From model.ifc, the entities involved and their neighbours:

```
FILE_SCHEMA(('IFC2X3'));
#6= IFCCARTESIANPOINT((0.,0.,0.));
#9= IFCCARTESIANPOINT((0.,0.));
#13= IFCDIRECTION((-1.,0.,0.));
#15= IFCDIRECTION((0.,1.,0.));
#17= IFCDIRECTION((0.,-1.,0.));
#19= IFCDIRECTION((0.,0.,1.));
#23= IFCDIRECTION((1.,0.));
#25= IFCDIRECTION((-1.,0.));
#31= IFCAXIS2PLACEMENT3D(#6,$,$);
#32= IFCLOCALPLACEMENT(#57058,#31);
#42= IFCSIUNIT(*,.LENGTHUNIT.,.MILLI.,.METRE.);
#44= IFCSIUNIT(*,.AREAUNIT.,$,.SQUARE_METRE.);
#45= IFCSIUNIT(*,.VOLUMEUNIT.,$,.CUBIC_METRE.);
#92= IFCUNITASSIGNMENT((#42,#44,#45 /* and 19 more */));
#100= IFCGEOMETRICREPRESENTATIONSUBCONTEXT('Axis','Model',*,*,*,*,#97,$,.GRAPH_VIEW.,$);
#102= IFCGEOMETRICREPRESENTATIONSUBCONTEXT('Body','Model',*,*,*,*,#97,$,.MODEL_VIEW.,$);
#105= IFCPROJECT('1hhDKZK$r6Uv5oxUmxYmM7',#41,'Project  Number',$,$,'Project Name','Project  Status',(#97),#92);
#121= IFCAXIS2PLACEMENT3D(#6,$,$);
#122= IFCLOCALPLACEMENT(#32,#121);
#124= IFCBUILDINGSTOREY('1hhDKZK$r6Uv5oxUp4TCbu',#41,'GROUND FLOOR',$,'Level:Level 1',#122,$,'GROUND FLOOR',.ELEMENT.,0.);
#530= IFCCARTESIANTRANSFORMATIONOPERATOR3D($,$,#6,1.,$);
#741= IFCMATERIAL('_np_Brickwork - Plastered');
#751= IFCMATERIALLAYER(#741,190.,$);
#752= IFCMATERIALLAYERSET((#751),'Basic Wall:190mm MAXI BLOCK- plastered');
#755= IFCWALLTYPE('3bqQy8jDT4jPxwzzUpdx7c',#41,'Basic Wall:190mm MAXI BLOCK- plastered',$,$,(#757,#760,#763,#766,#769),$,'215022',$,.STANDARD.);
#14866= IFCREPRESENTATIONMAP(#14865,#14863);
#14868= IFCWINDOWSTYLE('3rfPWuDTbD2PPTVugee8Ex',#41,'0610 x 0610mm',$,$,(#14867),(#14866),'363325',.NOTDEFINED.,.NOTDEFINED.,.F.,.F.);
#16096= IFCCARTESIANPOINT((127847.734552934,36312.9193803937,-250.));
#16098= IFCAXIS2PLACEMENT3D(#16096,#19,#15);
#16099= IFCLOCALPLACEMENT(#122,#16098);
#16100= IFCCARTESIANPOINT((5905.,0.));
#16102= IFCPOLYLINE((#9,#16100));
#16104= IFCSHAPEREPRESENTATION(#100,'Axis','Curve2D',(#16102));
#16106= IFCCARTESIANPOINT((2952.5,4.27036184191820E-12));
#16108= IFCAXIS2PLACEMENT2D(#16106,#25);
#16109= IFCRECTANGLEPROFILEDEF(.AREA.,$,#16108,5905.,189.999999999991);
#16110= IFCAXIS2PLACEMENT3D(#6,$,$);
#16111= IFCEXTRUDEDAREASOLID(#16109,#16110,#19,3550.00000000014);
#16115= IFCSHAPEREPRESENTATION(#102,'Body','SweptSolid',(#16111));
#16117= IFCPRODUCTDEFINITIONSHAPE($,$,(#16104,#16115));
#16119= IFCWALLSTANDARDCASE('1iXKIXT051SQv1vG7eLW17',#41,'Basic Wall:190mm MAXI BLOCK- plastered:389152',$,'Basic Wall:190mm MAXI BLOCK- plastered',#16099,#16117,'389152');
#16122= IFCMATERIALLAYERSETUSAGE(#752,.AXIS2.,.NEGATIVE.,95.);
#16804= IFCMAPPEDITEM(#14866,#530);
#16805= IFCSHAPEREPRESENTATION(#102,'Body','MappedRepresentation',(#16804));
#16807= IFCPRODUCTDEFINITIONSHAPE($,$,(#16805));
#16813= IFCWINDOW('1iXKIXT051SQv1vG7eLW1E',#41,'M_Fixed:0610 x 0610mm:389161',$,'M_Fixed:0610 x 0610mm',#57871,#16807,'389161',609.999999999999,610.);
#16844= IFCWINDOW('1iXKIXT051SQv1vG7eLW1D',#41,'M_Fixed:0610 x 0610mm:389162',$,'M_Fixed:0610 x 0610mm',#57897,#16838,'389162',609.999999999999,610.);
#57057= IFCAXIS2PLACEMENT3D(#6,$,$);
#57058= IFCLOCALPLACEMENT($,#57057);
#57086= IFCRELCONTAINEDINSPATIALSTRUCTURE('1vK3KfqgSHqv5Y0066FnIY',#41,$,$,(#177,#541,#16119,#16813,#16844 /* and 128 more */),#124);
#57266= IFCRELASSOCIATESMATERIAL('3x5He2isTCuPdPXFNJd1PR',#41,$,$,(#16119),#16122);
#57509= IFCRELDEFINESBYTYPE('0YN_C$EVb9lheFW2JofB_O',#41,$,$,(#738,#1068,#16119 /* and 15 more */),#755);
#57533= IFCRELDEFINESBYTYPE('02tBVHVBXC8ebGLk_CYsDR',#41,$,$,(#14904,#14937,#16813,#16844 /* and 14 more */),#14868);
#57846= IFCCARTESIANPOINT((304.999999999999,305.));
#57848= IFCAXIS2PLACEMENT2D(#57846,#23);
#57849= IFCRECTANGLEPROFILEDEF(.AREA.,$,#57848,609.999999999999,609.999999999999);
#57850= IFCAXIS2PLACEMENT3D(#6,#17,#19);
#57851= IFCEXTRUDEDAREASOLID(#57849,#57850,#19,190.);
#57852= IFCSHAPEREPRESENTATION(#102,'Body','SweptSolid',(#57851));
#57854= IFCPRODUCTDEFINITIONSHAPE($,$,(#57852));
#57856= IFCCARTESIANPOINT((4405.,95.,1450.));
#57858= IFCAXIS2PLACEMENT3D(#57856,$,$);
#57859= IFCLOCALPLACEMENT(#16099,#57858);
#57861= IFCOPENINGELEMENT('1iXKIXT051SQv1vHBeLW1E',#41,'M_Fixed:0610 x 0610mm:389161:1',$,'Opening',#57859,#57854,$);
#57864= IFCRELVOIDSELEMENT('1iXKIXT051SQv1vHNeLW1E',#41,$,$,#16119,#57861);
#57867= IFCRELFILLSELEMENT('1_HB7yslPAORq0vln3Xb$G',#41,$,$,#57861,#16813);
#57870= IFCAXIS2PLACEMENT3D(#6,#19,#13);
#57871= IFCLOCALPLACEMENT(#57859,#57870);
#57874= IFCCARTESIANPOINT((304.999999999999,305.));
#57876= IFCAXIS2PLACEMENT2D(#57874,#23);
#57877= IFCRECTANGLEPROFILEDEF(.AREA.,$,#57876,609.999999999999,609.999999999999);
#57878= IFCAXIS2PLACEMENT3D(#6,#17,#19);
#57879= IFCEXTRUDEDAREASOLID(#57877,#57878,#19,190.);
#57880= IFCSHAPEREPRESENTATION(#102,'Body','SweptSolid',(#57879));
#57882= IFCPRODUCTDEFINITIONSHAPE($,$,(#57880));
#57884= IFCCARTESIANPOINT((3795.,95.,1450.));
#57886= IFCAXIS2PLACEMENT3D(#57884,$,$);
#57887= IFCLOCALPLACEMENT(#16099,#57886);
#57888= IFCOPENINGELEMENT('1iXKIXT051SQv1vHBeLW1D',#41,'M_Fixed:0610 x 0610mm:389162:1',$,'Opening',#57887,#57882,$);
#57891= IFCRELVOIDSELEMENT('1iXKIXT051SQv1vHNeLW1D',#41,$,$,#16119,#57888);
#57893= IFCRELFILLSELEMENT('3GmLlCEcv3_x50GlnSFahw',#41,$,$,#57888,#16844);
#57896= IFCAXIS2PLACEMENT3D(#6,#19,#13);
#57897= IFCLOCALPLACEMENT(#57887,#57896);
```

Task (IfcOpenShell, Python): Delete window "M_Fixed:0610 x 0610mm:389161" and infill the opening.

```python
import ifcopenshell
import ifcopenshell.api.feature
import ifcopenshell.api.root
import ifcopenshell.geom
import ifcopenshell.util.shape

model = ifcopenshell.open("model.ifc")
settings = ifcopenshell.geom.settings()


def volume(element):
    """Net volume in cubic metres, openings subtracted."""
    shape = ifcopenshell.geom.create_shape(settings, element)
    return ifcopenshell.util.shape.get_volume(shape.geometry)


window = model.by_guid("1iXKIXT051SQv1vG7eLW1E")
opening = window.FillsVoids[0].RelatingOpeningElement
wall = opening.VoidsElements[0].RelatingBuildingElement
before = volume(wall)

ifcopenshell.api.root.remove_product(model, product=window)
ifcopenshell.api.feature.remove_feature(model, feature=opening)

after = volume(wall)

print(f"wall volume {before:.3f} -> {after:.3f} m3")

model.write("model-out.ifc")
```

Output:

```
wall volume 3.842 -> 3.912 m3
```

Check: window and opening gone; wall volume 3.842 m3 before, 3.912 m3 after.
